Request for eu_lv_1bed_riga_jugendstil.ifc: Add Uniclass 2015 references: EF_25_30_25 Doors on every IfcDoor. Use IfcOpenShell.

First a look at what the model holds.

```python
import ifcopenshell

model = ifcopenshell.open("eu_lv_1bed_riga_jugendstil.ifc")
print(model.schema)
print("classifications:", [c.Name for c in model.by_type("IfcClassification")])
for ifc_class in ("IfcDoor", "IfcRoof", "IfcStair", "IfcWall", "IfcWindow"):
    print(ifc_class, len(model.by_type(ifc_class)))
```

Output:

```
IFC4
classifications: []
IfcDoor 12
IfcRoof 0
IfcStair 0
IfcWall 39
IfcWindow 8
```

```python
import ifcopenshell
import ifcopenshell.api.classification

model = ifcopenshell.open("eu_lv_1bed_riga_jugendstil.ifc")

system = ifcopenshell.api.classification.add_classification(model, classification="Uniclass 2015")

codes = {
    "IfcDoor": ("EF_25_30_25", "Doors"),
}
for ifc_class, (code, name) in codes.items():
    products = model.by_type(ifc_class)
    ifcopenshell.api.classification.add_reference(
        model, products=products, classification=system, identification=code, name=name
    )
    print(code, len(products))

model.write("eu_lv_1bed_riga_jugendstil_updated.ifc")
```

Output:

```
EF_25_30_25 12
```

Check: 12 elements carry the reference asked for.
